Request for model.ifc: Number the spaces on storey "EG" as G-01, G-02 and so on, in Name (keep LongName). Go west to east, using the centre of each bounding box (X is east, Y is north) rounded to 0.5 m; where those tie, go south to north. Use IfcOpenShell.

First a look at what the model holds.

```python
import ifcopenshell
import ifcopenshell.util.element
import ifcopenshell.util.placement

model = ifcopenshell.open("model.ifc")
print(model.schema)
storey = next(s for s in model.by_type("IfcBuildingStorey") if s.Name == "EG")
spaces = [e for e in ifcopenshell.util.element.get_decomposition(storey) if e.is_a("IfcSpace")]
for e in sorted(spaces, key=lambda e: e.id()):
    origin = ifcopenshell.util.placement.get_local_placement(e.ObjectPlacement)[:3, 3]
    print(e.id(), e.Name, e.LongName, origin.round(2) + 0.0, sep=" | ")
```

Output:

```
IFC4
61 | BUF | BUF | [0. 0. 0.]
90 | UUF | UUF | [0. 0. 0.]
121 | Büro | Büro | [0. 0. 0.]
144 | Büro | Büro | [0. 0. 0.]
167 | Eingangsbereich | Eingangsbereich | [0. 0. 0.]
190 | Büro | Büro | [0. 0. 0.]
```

```python
import ifcopenshell
import ifcopenshell.geom
import ifcopenshell.util.element
import ifcopenshell.util.shape

model = ifcopenshell.open("model.ifc")
settings = ifcopenshell.geom.settings()
settings.set("use-world-coords", True)


def centre(element):
    shape = ifcopenshell.geom.create_shape(settings, element)
    return ifcopenshell.util.shape.get_bbox_centroid(shape.geometry)


storey = next(s for s in model.by_type("IfcBuildingStorey") if s.Name == "EG")
spaces = [e for e in ifcopenshell.util.element.get_decomposition(storey) if e.is_a("IfcSpace")]

# Insertion points can sit at a corner or the storey origin, so sort by the geometry (in metres).
centres = {e: centre(e) for e in spaces}
spaces.sort(key=lambda e: (round(centres[e][0] / 0.5), centres[e][1]))

for i, e in enumerate(spaces, start=1):
    number = f"G-{i:02d}"
    e.Name = number
    print(e.id(), number)

model.write("model-out.ifc")
```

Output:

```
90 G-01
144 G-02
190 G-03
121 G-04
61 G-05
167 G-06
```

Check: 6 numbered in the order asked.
